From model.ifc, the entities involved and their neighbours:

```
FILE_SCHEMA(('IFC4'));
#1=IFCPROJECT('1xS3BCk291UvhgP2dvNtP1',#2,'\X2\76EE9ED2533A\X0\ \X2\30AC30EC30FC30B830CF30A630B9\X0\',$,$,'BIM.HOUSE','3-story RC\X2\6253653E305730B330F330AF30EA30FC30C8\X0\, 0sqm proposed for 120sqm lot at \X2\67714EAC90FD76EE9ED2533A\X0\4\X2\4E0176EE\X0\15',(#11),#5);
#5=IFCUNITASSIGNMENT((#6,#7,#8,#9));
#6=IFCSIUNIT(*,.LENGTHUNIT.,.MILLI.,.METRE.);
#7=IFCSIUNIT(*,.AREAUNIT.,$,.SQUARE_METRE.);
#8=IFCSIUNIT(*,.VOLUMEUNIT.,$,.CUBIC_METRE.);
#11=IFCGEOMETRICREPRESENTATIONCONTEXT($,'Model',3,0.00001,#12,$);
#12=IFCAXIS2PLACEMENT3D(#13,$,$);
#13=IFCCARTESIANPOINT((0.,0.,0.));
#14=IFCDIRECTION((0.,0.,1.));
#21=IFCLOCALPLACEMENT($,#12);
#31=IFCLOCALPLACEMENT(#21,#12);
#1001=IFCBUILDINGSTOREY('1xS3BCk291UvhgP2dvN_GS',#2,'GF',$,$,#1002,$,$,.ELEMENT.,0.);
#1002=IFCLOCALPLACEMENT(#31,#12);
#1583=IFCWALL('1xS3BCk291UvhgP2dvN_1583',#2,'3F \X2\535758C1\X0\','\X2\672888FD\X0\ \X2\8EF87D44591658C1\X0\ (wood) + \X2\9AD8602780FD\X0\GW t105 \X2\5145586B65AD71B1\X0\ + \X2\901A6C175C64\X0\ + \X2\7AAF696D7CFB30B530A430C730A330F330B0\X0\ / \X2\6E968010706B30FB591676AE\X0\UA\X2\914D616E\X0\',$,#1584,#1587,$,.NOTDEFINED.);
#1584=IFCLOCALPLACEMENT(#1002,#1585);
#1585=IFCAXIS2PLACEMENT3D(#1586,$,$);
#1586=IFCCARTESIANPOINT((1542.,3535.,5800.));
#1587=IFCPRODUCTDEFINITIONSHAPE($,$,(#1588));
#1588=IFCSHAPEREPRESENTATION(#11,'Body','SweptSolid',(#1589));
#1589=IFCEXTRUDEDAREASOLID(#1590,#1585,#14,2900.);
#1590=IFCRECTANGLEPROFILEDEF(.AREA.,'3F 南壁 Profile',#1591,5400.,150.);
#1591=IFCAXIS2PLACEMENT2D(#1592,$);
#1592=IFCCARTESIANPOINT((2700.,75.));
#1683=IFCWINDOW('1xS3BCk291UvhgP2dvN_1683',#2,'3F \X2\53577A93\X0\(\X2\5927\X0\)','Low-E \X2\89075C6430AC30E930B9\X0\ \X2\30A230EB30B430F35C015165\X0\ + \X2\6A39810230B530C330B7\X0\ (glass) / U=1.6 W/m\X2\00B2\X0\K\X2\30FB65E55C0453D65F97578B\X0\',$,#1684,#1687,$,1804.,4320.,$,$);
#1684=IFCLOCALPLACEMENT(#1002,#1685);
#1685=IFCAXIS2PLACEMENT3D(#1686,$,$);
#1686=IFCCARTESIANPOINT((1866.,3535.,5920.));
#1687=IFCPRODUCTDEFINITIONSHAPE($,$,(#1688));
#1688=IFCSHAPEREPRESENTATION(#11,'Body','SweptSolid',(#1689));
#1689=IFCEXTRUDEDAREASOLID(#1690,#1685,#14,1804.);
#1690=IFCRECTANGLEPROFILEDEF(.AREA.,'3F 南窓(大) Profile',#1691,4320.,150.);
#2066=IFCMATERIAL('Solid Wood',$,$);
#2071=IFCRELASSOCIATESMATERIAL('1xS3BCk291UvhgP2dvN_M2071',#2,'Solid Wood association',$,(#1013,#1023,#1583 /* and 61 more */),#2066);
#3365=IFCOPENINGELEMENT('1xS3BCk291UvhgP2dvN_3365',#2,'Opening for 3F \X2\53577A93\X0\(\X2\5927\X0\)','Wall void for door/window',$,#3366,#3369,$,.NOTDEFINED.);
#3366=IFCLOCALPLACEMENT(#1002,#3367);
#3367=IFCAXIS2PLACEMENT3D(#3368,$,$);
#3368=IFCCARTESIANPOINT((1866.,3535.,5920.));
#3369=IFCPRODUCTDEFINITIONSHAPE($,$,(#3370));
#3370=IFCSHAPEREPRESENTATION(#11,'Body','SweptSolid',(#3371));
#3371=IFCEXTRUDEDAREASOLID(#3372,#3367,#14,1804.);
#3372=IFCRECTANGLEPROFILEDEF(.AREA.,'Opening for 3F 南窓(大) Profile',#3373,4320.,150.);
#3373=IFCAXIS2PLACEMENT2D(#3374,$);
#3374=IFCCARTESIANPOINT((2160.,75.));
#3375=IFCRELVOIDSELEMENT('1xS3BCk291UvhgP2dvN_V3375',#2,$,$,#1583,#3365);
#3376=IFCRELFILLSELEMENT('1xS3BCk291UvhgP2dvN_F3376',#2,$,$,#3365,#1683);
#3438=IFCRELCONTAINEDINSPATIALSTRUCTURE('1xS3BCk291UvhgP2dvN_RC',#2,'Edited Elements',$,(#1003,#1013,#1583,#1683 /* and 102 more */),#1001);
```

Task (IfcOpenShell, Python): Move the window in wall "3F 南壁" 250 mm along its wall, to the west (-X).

```python
import ifcopenshell
import ifcopenshell.api.geometry
import ifcopenshell.util.placement
import ifcopenshell.util.unit

model = ifcopenshell.open("model.ifc")
unit_scale = ifcopenshell.util.unit.calculate_unit_scale(model)

window = model.by_guid("1xS3BCk291UvhgP2dvN_1683")
opening = window.FillsVoids[0].RelatingOpeningElement
wall = opening.VoidsElements[0].RelatingBuildingElement

wall_matrix = ifcopenshell.util.placement.get_local_placement(wall.ObjectPlacement)
shift = wall_matrix[:3, 0] * -0.25 / unit_scale
before = ifcopenshell.util.placement.get_local_placement(window.ObjectPlacement)[:3, 3].copy()

# The window is not placed relative to its opening, so move both.
for product in (opening, window):
    matrix = ifcopenshell.util.placement.get_local_placement(product.ObjectPlacement)
    matrix[:3, 3] += shift
    ifcopenshell.api.geometry.edit_object_placement(model, product=product, matrix=matrix, is_si=False)

after = ifcopenshell.util.placement.get_local_placement(window.ObjectPlacement)[:3, 3]
print("window moved by", (after - before).round(3) + 0.0)

model.write("model_v2.ifc")
```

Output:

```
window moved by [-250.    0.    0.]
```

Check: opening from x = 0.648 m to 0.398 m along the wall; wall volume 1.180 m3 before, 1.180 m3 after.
